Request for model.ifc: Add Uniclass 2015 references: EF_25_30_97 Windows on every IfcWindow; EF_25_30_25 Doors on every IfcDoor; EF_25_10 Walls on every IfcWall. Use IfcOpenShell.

First a look at what the model holds.

```python
import ifcopenshell

model = ifcopenshell.open("model.ifc")
print(model.schema)
print("classifications:", [c.Name for c in model.by_type("IfcClassification")])
for ifc_class in ("IfcDoor", "IfcRoof", "IfcStair", "IfcWall", "IfcWindow"):
    print(ifc_class, len(model.by_type(ifc_class)))
```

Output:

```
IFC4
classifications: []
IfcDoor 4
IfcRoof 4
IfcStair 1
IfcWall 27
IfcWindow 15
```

```python
import ifcopenshell
import ifcopenshell.api.classification

model = ifcopenshell.open("model.ifc")

system = ifcopenshell.api.classification.add_classification(model, classification="Uniclass 2015")

codes = {
    "IfcWindow": ("EF_25_30_97", "Windows"),
    "IfcDoor": ("EF_25_30_25", "Doors"),
    "IfcWall": ("EF_25_10", "Walls"),
}
for ifc_class, (code, name) in codes.items():
    products = model.by_type(ifc_class)
    ifcopenshell.api.classification.add_reference(
        model, products=products, classification=system, identification=code, name=name
    )
    print(code, len(products))

model.write("model_v2.ifc")
```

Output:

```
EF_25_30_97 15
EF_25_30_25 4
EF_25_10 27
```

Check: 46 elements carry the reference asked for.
